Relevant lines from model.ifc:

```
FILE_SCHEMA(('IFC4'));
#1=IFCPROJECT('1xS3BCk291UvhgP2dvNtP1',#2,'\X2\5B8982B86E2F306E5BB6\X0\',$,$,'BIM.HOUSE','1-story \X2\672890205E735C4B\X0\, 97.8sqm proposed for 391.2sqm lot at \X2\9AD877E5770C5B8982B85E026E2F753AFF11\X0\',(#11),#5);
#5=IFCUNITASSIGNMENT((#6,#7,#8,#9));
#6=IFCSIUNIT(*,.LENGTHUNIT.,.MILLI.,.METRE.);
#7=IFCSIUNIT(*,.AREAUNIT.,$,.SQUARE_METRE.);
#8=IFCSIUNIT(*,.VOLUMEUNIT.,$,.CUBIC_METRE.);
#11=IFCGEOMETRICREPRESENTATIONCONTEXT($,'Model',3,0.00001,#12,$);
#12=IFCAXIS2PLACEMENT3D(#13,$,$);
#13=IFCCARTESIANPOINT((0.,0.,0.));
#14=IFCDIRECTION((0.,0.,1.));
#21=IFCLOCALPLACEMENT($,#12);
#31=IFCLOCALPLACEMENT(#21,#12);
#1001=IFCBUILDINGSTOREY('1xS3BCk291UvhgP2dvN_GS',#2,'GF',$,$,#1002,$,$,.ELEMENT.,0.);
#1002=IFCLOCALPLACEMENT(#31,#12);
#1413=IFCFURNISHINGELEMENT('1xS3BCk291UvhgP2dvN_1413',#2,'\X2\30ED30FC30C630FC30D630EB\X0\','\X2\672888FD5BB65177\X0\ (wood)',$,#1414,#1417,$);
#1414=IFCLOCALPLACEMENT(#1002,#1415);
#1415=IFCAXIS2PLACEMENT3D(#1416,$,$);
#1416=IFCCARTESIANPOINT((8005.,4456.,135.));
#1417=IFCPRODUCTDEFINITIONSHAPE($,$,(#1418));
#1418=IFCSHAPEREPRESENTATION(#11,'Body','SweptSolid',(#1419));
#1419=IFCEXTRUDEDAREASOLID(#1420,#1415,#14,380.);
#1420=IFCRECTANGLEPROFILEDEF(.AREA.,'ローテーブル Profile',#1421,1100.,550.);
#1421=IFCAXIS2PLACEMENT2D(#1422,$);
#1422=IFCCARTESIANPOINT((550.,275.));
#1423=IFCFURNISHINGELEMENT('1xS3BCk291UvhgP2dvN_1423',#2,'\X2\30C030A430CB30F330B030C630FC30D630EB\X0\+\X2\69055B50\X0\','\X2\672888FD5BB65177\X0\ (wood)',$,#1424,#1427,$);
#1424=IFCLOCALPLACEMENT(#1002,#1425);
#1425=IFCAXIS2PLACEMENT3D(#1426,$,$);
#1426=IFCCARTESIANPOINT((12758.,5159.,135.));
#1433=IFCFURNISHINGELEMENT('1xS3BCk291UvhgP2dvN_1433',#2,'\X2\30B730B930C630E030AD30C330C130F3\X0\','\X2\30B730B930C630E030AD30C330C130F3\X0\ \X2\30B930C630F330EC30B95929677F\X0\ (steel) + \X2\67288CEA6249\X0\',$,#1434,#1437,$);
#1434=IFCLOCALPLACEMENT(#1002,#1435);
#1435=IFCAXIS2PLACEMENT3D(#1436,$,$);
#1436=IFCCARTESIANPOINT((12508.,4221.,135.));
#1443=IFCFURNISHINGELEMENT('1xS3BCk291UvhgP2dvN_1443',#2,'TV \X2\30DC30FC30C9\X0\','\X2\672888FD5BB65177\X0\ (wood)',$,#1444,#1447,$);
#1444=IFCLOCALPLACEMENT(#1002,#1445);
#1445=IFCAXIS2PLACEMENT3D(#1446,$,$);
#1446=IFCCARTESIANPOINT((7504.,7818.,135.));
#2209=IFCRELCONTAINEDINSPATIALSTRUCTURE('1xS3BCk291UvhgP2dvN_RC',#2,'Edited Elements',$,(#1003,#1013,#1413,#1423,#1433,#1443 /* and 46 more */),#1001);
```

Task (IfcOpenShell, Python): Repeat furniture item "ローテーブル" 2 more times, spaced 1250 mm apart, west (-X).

```python
import numpy as np
import ifcopenshell
import ifcopenshell.api.geometry
import ifcopenshell.api.root
import ifcopenshell.util.element
import ifcopenshell.util.placement
import ifcopenshell.util.unit

model = ifcopenshell.open("model.ifc")
unit_scale = ifcopenshell.util.unit.calculate_unit_scale(model)


def reuse_history(source, copy):
    """copy_class also copies each property set's owner history, people and application; keep the originals."""
    for rel in copy.IsDefinedBy:
        if rel.is_a("IfcRelDefinesByProperties") and (history := rel.RelatingPropertyDefinition.OwnerHistory):
            rel.RelatingPropertyDefinition.OwnerHistory = source.OwnerHistory
            ifcopenshell.util.element.remove_deep2(model, history)


source = model.by_guid("1xS3BCk291UvhgP2dvN_1413")
base = ifcopenshell.util.placement.get_local_placement(source.ObjectPlacement)
step = np.array([-1.0, 0.0, 0.0]) * 1.25 / unit_scale

for i in range(1, 3):
    copy = ifcopenshell.api.root.copy_class(model, product=source)
    copy.Representation = ifcopenshell.util.element.copy_deep(
        model, source.Representation, exclude=["IfcGeometricRepresentationContext", "IfcRepresentationMap"]
    )
    reuse_history(source, copy)
    matrix = base.copy()
    matrix[:3, 3] += i * step
    print("added at", matrix[:3, 3].round(3) + 0.0)
    ifcopenshell.api.geometry.edit_object_placement(model, product=copy, matrix=matrix, is_si=False)

model.write("model-out.ifc")
```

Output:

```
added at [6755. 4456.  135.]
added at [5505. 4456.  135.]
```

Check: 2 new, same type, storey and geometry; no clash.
